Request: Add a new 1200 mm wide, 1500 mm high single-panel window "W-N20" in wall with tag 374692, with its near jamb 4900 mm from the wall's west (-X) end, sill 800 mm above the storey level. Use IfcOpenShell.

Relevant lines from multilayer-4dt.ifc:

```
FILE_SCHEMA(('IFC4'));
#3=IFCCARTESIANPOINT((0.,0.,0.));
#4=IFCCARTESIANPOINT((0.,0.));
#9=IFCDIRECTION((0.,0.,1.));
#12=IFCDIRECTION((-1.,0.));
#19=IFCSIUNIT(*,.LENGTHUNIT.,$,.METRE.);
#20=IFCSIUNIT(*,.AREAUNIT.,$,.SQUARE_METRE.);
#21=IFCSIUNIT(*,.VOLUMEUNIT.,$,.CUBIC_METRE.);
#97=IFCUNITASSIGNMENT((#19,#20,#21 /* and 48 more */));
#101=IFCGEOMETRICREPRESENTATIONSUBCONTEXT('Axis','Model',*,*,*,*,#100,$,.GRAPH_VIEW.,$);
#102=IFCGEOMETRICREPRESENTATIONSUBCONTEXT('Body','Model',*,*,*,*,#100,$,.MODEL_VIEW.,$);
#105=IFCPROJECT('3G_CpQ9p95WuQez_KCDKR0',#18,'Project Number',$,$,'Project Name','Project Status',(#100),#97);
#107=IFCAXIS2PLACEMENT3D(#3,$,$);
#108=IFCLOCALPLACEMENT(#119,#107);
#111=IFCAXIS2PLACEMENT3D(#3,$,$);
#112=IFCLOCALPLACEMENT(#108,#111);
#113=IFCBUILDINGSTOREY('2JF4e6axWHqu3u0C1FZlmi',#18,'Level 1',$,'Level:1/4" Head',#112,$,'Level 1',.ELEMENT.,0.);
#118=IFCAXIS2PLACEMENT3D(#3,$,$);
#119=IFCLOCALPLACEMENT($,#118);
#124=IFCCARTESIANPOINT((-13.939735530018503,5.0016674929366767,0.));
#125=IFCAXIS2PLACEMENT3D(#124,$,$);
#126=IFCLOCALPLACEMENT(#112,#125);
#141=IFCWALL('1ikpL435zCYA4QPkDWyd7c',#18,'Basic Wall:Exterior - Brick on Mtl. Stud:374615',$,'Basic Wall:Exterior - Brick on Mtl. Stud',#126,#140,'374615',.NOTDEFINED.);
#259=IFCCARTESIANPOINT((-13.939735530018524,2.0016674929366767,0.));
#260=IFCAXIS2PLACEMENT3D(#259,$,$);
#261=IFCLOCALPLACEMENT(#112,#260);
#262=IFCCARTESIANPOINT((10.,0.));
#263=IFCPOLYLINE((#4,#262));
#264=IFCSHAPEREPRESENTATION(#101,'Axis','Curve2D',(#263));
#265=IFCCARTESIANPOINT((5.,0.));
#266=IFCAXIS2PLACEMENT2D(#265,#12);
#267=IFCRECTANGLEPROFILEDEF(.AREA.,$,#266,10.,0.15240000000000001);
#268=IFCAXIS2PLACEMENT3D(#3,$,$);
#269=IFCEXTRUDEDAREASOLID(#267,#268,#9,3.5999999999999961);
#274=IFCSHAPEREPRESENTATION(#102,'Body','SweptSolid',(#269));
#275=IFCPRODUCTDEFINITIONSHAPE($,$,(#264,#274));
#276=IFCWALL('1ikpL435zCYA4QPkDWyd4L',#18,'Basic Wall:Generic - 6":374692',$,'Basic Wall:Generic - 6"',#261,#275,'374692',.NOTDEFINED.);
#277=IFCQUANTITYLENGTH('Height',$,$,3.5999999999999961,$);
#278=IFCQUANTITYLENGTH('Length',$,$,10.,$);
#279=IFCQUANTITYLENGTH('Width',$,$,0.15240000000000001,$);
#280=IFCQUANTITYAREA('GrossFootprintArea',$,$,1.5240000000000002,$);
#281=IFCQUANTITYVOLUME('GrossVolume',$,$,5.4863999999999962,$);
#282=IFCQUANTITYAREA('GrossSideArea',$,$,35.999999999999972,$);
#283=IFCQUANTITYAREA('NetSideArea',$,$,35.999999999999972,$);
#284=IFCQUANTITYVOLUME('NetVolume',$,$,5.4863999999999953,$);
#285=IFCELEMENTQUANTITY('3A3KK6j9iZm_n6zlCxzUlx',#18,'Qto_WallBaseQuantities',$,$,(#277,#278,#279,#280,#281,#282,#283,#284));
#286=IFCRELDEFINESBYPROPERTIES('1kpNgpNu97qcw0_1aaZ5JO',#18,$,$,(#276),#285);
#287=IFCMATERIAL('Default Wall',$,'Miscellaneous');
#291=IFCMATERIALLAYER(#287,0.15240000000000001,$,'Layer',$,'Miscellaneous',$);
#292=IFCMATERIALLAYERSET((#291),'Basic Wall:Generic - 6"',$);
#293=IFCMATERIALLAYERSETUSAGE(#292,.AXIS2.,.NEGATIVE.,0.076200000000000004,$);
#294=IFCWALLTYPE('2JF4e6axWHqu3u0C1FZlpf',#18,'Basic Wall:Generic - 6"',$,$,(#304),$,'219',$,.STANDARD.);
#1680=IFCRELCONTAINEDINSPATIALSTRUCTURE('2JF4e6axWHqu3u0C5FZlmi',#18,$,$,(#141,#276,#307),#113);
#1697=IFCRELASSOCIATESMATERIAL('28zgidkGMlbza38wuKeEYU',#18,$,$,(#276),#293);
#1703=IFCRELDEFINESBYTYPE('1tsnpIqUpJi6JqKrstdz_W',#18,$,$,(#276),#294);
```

```python
import numpy as np
import ifcopenshell
import ifcopenshell.api.feature
import ifcopenshell.api.geometry
import ifcopenshell.api.pset
import ifcopenshell.api.root
import ifcopenshell.api.spatial
import ifcopenshell.geom
import ifcopenshell.util.element
import ifcopenshell.util.placement
import ifcopenshell.util.representation
import ifcopenshell.util.shape
import ifcopenshell.util.unit

model = ifcopenshell.open("multilayer-4dt.ifc")
unit_scale = ifcopenshell.util.unit.calculate_unit_scale(model)
area_scale = ifcopenshell.util.unit.calculate_unit_scale(model, "AREAUNIT")
volume_scale = ifcopenshell.util.unit.calculate_unit_scale(model, "VOLUMEUNIT")
settings = ifcopenshell.geom.settings()


def volume(element):
    """Net volume in cubic metres, openings subtracted."""
    shape = ifcopenshell.geom.create_shape(settings, element)
    return ifcopenshell.util.shape.get_volume(shape.geometry)


wall = model.by_guid("1ikpL435zCYA4QPkDWyd4L")
storey = ifcopenshell.util.element.get_container(wall, ifc_class="IfcBuildingStorey")
context = ifcopenshell.util.representation.get_context(model, "Model", "Body", "MODEL_VIEW")
before = volume(wall)

width, height, from_end, sill = 1.2, 1.5, 4.9, 0.8  # metres

# The wall runs along its own X axis, and the end named is its -X end.
wall_shape = ifcopenshell.geom.create_shape(settings, wall)
x, y, z = ifcopenshell.util.shape.get_vertices(wall_shape.geometry).T
start = x.min() + from_end
face, thickness = float(y.min()), float(y.max() - y.min())
wall_matrix = ifcopenshell.util.placement.get_local_placement(wall.ObjectPlacement)
level = ifcopenshell.util.placement.get_local_placement(storey.ObjectPlacement)[2, 3]


def in_wall(x, y):
    """Placement at x, y metres in the wall's axes, at sill height."""
    matrix = wall_matrix.copy()
    matrix[:, 3] = wall_matrix @ np.array([x / unit_scale, y / unit_scale, 0.0, 1.0])
    matrix[2, 3] = level + sill / unit_scale
    return matrix


# Opening: a box that overshoots both wall faces by 50 mm.
opening = ifcopenshell.api.root.create_entity(model, ifc_class="IfcOpeningElement", predefined_type="OPENING")
box = ifcopenshell.api.geometry.add_wall_representation(
    model, context=context, length=width, height=height, thickness=thickness + 0.1
)
ifcopenshell.api.geometry.assign_representation(model, product=opening, representation=box)
ifcopenshell.api.geometry.edit_object_placement(model, product=opening, matrix=in_wall(start, face - 0.05), is_si=False)
ifcopenshell.api.feature.add_feature(model, feature=opening, element=wall)

window = ifcopenshell.api.root.create_entity(model, ifc_class="IfcWindow", name="W-N20", predefined_type="WINDOW")
window.OverallWidth, window.OverallHeight = width / unit_scale, height / unit_scale
window.PartitioningType = "SINGLE_PANEL"
body = ifcopenshell.api.geometry.add_window_representation(
    model,
    context=context,
    overall_width=window.OverallWidth,
    overall_height=window.OverallHeight,
    partition_type="SINGLE_PANEL",
)
ifcopenshell.api.geometry.assign_representation(model, product=window, representation=body)
ifcopenshell.api.spatial.assign_container(model, products=[window], relating_structure=storey)
ifcopenshell.api.feature.add_filling(model, opening=opening, element=window)

# Centre the window in the wall's thickness.
ifcopenshell.api.geometry.edit_object_placement(model, product=window, matrix=in_wall(start, face), is_si=False)
window_shape = ifcopenshell.geom.create_shape(settings, window)
depth = ifcopenshell.util.shape.get_vertices(window_shape.geometry)[:, 1]
offset = face + thickness / 2 - (depth.min() + depth.max()) / 2
ifcopenshell.api.geometry.edit_object_placement(model, product=window, matrix=in_wall(start, offset), is_si=False)

after = volume(wall)

# Update the wall's stored quantities.
qto = model.by_id(ifcopenshell.util.element.get_pset(wall, "Qto_WallBaseQuantities", should_inherit=False)["id"])
ifcopenshell.api.pset.edit_qto(model, qto=qto, properties={
    "NetSideArea": after / thickness / area_scale,
    "NetVolume": after / volume_scale,
})

print(f"wall volume {before:.3f} -> {after:.3f} m3")

model.write("multilayer-4dt-out.ifc")
```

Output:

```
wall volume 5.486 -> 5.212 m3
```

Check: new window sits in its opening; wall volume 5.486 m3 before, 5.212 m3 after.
